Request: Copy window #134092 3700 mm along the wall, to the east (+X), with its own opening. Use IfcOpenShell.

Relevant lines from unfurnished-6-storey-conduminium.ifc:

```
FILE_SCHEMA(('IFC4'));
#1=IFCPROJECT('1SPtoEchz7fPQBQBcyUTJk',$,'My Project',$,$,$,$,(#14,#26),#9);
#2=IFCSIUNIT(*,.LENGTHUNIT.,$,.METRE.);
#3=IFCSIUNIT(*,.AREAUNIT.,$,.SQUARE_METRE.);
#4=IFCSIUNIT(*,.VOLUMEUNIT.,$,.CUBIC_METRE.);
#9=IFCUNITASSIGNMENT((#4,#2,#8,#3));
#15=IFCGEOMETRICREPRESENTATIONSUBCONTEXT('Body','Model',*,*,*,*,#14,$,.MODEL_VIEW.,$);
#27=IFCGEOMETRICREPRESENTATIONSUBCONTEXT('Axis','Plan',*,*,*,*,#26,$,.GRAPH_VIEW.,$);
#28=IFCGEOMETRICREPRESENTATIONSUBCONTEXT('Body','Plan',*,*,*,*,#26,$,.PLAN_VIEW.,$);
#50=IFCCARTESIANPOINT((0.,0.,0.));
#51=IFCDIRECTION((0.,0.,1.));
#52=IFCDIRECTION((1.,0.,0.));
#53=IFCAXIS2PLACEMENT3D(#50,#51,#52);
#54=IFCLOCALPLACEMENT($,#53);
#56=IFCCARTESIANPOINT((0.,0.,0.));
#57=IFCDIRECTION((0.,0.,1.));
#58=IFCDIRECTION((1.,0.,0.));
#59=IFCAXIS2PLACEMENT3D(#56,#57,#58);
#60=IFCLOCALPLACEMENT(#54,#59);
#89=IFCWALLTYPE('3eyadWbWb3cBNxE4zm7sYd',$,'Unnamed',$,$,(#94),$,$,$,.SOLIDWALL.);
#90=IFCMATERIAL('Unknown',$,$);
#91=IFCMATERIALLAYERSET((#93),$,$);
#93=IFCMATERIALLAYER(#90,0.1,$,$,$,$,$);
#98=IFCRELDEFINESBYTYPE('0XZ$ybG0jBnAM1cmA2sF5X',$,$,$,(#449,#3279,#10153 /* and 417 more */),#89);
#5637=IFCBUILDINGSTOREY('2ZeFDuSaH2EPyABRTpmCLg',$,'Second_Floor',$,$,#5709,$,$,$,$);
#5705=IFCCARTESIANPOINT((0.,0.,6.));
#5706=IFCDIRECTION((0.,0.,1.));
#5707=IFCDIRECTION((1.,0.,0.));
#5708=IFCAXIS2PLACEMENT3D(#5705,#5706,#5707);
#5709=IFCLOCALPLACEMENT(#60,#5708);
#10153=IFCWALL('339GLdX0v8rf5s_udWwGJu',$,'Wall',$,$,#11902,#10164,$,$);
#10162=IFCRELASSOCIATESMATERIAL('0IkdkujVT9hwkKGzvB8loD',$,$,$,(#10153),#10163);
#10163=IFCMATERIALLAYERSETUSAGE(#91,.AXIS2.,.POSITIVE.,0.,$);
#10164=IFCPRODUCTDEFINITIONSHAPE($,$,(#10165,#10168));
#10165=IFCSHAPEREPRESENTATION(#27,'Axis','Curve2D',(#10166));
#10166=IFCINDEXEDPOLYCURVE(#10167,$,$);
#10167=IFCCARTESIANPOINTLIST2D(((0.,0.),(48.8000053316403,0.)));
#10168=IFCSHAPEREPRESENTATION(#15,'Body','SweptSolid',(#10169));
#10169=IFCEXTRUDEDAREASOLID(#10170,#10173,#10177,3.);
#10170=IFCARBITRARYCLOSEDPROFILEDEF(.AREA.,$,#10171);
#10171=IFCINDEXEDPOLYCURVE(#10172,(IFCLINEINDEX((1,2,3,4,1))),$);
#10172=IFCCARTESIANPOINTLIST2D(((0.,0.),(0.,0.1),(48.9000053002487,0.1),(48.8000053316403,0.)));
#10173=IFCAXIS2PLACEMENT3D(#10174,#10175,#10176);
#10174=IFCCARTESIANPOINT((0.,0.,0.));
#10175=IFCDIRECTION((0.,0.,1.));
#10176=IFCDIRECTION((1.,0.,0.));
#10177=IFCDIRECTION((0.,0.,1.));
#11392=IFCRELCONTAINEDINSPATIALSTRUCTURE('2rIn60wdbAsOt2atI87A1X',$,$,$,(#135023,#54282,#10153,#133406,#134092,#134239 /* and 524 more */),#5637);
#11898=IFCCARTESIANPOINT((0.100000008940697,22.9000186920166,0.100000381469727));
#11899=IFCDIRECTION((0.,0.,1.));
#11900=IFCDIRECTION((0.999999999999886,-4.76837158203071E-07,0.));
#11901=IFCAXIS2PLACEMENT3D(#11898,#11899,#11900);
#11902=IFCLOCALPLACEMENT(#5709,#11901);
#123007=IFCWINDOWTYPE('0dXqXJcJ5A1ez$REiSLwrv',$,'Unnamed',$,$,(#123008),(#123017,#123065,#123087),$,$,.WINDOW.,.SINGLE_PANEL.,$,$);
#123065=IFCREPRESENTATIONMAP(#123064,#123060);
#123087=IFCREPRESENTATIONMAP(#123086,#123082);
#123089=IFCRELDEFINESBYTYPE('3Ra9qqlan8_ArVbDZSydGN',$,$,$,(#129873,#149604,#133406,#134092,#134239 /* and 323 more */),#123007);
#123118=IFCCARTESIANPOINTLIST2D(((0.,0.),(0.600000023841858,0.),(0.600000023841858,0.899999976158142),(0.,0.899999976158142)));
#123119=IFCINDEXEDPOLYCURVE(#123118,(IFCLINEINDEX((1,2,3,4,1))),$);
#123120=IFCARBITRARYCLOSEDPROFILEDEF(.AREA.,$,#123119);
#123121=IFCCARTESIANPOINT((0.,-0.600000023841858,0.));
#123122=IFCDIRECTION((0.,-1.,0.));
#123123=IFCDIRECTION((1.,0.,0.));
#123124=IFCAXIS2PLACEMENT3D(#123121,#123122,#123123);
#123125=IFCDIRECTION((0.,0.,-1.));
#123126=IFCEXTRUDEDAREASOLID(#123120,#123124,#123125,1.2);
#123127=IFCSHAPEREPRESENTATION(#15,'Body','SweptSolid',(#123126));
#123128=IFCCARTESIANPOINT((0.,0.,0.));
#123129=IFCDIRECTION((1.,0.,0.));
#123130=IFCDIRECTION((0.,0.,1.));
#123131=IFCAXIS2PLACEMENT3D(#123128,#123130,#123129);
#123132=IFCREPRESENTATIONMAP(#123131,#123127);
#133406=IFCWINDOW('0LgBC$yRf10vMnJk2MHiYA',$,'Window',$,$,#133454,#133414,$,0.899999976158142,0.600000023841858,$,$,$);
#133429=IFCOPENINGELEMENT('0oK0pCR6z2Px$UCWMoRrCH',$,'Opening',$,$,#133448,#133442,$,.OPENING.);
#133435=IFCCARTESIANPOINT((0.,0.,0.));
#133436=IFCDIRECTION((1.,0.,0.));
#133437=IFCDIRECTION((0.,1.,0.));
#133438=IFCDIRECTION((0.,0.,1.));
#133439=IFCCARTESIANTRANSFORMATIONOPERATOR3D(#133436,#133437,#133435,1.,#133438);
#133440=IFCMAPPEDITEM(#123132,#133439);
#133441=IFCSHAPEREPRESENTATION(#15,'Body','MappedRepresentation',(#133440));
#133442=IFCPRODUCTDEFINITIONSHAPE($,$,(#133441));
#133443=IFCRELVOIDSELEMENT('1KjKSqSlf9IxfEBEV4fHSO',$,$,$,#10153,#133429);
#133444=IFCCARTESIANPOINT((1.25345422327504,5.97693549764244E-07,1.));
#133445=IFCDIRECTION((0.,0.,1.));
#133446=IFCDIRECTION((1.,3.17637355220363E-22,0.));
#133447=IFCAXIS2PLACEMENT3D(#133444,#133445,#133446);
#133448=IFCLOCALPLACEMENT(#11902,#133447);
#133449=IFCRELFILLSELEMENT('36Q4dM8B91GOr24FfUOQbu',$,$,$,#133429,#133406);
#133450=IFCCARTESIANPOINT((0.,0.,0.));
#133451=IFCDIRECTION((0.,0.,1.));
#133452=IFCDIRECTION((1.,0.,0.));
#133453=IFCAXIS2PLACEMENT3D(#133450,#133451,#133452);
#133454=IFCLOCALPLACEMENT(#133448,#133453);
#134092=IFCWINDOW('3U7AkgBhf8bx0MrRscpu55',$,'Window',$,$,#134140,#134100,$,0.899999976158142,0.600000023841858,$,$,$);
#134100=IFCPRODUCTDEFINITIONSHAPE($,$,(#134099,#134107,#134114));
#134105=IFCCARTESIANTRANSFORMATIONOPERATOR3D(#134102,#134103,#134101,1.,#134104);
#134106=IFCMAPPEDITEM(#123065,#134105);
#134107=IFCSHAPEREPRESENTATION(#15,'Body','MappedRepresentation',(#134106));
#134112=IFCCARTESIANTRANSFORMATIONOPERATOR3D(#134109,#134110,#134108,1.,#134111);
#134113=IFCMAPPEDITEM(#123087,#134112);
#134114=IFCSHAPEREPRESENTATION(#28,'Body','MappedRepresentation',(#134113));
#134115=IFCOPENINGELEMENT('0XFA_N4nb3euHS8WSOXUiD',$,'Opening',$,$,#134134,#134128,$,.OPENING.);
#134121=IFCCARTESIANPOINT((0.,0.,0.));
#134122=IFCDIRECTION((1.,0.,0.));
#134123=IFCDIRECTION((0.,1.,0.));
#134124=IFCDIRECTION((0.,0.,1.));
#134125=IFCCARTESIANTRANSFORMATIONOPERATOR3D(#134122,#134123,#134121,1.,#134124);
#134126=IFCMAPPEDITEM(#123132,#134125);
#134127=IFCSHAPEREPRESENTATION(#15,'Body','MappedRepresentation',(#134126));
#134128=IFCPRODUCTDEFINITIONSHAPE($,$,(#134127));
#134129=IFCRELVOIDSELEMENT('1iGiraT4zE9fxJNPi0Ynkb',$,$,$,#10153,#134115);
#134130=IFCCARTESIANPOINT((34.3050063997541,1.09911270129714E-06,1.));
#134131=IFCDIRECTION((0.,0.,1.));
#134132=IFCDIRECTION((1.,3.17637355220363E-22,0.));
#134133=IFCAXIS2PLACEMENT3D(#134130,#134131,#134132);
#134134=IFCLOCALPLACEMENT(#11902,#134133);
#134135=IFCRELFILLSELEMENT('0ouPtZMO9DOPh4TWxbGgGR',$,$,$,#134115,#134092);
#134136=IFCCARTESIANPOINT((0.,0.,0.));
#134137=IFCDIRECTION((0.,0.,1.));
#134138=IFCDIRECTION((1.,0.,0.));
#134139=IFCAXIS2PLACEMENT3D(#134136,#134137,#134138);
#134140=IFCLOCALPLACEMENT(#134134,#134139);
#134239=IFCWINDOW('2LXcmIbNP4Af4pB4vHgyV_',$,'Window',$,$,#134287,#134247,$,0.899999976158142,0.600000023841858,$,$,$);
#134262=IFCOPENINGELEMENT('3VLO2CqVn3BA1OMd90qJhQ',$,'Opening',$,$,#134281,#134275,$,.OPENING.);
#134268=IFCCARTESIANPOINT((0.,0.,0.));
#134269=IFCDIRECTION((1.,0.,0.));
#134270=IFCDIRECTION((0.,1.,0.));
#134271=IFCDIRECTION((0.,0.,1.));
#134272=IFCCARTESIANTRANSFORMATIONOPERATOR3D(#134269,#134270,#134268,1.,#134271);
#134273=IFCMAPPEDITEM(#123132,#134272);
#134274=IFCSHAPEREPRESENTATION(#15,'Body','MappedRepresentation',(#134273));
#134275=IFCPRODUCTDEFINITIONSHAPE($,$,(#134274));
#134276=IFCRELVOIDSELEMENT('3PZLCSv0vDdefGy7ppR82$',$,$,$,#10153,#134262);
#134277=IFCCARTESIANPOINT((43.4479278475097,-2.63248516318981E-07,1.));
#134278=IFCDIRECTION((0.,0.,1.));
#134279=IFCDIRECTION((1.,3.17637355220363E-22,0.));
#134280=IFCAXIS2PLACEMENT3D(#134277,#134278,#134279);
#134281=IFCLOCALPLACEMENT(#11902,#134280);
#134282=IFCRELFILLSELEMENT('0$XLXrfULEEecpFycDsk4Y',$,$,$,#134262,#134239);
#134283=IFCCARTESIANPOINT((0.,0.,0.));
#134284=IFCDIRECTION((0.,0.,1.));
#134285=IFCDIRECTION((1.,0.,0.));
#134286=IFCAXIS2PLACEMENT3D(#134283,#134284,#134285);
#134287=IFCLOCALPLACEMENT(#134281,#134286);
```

```python
import ifcopenshell
import ifcopenshell.api.feature
import ifcopenshell.api.geometry
import ifcopenshell.api.root
import ifcopenshell.geom
import ifcopenshell.util.element
import ifcopenshell.util.placement
import ifcopenshell.util.shape
import ifcopenshell.util.unit

model = ifcopenshell.open("unfurnished-6-storey-conduminium.ifc")
unit_scale = ifcopenshell.util.unit.calculate_unit_scale(model)
settings = ifcopenshell.geom.settings()


def volume(element):
    """Net volume in cubic metres, openings subtracted."""
    shape = ifcopenshell.geom.create_shape(settings, element)
    return ifcopenshell.util.shape.get_volume(shape.geometry)


window = model.by_guid("3U7AkgBhf8bx0MrRscpu55")
opening = window.FillsVoids[0].RelatingOpeningElement
wall = opening.VoidsElements[0].RelatingBuildingElement
before = volume(wall)
shift = ifcopenshell.util.placement.get_local_placement(wall.ObjectPlacement)[:3, 0] * 3.7 / unit_scale

# copy_class copies the void relationship, type, container and properties, but no geometry.
new_opening = ifcopenshell.api.root.copy_class(model, product=opening)
new_opening.Representation = ifcopenshell.util.element.copy_deep(
    model, opening.Representation, exclude=["IfcGeometricRepresentationContext", "IfcRepresentationMap"]
)
new_window = ifcopenshell.api.root.copy_class(model, product=window)
new_window.Representation = ifcopenshell.util.element.copy_deep(
    model, window.Representation, exclude=["IfcGeometricRepresentationContext", "IfcRepresentationMap"]
)
ifcopenshell.api.feature.add_filling(model, opening=new_opening, element=new_window)

for old, new in ((opening, new_opening), (window, new_window)):
    matrix = ifcopenshell.util.placement.get_local_placement(old.ObjectPlacement)
    matrix[:3, 3] += shift
    ifcopenshell.api.geometry.edit_object_placement(model, product=new, matrix=matrix, is_si=False)

after = volume(wall)

print(f"wall volume {before:.3f} -> {after:.3f} m3")

model.write("unfurnished-6-storey-conduminium_rev.ifc")
```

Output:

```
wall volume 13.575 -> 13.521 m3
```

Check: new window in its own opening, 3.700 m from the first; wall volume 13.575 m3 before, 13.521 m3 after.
